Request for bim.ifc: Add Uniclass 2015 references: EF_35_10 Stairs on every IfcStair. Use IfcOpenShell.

First a look at what the model holds.

```python
import ifcopenshell

model = ifcopenshell.open("bim.ifc")
print(model.schema)
print("classifications:", [c.Name for c in model.by_type("IfcClassification")])
for ifc_class in ("IfcDoor", "IfcRoof", "IfcStair", "IfcWall", "IfcWindow"):
    print(ifc_class, len(model.by_type(ifc_class)))
```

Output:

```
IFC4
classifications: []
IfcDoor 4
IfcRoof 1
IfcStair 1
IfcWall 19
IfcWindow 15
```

```python
import ifcopenshell
import ifcopenshell.api.classification

model = ifcopenshell.open("bim.ifc")

system = ifcopenshell.api.classification.add_classification(model, classification="Uniclass 2015")

codes = {
    "IfcStair": ("EF_35_10", "Stairs"),
}
for ifc_class, (code, name) in codes.items():
    products = model.by_type(ifc_class)
    ifcopenshell.api.classification.add_reference(
        model, products=products, classification=system, identification=code, name=name
    )
    print(code, len(products))

model.write("bim_v2.ifc")
```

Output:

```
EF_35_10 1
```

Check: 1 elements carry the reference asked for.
